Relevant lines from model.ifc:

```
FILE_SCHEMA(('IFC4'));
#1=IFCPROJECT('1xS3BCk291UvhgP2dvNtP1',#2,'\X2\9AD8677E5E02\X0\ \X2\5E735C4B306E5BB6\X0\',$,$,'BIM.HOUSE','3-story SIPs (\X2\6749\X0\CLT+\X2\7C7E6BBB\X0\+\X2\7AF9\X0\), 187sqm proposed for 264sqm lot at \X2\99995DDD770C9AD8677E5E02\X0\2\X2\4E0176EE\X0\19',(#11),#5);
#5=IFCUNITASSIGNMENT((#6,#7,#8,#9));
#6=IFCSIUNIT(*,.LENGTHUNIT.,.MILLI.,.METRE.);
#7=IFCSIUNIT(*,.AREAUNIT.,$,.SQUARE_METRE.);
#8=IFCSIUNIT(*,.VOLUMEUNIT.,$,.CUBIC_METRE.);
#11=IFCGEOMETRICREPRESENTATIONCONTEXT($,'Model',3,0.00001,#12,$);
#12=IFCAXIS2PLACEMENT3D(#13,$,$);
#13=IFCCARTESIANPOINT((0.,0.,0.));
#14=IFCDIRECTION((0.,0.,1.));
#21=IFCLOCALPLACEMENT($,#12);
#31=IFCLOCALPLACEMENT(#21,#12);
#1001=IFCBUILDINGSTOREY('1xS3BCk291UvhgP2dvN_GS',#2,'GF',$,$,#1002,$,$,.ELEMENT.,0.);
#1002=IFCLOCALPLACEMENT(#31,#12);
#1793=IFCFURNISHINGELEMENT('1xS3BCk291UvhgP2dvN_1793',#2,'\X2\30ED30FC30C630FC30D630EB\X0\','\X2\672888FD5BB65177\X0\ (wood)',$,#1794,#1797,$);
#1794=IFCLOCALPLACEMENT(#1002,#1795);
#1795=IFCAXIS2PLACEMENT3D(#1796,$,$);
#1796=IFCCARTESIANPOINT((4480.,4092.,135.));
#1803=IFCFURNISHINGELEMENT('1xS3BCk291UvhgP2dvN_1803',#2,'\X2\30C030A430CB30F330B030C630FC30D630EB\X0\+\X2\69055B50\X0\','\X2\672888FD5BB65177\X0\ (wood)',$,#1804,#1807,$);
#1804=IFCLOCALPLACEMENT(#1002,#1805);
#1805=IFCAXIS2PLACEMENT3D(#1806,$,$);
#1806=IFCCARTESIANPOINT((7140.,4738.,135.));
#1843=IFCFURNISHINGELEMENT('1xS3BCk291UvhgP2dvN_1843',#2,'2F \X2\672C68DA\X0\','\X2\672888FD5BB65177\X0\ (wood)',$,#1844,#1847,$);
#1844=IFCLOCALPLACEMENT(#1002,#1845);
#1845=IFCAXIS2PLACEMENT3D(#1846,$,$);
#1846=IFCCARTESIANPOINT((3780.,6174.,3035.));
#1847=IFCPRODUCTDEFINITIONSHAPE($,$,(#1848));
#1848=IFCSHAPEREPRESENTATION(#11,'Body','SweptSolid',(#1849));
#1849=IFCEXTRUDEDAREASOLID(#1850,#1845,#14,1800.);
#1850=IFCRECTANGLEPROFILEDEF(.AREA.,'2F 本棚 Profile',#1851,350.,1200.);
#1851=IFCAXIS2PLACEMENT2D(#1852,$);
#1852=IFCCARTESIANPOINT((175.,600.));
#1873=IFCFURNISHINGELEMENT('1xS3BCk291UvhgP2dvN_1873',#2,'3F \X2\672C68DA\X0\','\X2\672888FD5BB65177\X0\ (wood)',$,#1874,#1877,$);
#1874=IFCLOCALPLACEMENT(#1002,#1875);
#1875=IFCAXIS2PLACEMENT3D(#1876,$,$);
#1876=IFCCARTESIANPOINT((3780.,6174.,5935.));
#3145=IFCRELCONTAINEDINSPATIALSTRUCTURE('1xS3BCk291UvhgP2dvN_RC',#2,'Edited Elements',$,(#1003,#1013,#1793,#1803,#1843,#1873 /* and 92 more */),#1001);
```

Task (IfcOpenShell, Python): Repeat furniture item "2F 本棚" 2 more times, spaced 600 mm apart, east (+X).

```python
import numpy as np
import ifcopenshell
import ifcopenshell.api.geometry
import ifcopenshell.api.root
import ifcopenshell.util.element
import ifcopenshell.util.placement
import ifcopenshell.util.unit

model = ifcopenshell.open("model.ifc")
unit_scale = ifcopenshell.util.unit.calculate_unit_scale(model)


def reuse_history(source, copy):
    """copy_class also copies each property set's owner history, people and application; keep the originals."""
    for rel in copy.IsDefinedBy:
        if rel.is_a("IfcRelDefinesByProperties") and (history := rel.RelatingPropertyDefinition.OwnerHistory):
            rel.RelatingPropertyDefinition.OwnerHistory = source.OwnerHistory
            ifcopenshell.util.element.remove_deep2(model, history)


source = model.by_guid("1xS3BCk291UvhgP2dvN_1843")
base = ifcopenshell.util.placement.get_local_placement(source.ObjectPlacement)
step = np.array([1.0, 0.0, 0.0]) * 0.6 / unit_scale

for i in range(1, 3):
    copy = ifcopenshell.api.root.copy_class(model, product=source)
    copy.Representation = ifcopenshell.util.element.copy_deep(
        model, source.Representation, exclude=["IfcGeometricRepresentationContext", "IfcRepresentationMap"]
    )
    reuse_history(source, copy)
    matrix = base.copy()
    matrix[:3, 3] += i * step
    print("added at", matrix[:3, 3].round(3) + 0.0)
    ifcopenshell.api.geometry.edit_object_placement(model, product=copy, matrix=matrix, is_si=False)

model.write("model-out.ifc")
```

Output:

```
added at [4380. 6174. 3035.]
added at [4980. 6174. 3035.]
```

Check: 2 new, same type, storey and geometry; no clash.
